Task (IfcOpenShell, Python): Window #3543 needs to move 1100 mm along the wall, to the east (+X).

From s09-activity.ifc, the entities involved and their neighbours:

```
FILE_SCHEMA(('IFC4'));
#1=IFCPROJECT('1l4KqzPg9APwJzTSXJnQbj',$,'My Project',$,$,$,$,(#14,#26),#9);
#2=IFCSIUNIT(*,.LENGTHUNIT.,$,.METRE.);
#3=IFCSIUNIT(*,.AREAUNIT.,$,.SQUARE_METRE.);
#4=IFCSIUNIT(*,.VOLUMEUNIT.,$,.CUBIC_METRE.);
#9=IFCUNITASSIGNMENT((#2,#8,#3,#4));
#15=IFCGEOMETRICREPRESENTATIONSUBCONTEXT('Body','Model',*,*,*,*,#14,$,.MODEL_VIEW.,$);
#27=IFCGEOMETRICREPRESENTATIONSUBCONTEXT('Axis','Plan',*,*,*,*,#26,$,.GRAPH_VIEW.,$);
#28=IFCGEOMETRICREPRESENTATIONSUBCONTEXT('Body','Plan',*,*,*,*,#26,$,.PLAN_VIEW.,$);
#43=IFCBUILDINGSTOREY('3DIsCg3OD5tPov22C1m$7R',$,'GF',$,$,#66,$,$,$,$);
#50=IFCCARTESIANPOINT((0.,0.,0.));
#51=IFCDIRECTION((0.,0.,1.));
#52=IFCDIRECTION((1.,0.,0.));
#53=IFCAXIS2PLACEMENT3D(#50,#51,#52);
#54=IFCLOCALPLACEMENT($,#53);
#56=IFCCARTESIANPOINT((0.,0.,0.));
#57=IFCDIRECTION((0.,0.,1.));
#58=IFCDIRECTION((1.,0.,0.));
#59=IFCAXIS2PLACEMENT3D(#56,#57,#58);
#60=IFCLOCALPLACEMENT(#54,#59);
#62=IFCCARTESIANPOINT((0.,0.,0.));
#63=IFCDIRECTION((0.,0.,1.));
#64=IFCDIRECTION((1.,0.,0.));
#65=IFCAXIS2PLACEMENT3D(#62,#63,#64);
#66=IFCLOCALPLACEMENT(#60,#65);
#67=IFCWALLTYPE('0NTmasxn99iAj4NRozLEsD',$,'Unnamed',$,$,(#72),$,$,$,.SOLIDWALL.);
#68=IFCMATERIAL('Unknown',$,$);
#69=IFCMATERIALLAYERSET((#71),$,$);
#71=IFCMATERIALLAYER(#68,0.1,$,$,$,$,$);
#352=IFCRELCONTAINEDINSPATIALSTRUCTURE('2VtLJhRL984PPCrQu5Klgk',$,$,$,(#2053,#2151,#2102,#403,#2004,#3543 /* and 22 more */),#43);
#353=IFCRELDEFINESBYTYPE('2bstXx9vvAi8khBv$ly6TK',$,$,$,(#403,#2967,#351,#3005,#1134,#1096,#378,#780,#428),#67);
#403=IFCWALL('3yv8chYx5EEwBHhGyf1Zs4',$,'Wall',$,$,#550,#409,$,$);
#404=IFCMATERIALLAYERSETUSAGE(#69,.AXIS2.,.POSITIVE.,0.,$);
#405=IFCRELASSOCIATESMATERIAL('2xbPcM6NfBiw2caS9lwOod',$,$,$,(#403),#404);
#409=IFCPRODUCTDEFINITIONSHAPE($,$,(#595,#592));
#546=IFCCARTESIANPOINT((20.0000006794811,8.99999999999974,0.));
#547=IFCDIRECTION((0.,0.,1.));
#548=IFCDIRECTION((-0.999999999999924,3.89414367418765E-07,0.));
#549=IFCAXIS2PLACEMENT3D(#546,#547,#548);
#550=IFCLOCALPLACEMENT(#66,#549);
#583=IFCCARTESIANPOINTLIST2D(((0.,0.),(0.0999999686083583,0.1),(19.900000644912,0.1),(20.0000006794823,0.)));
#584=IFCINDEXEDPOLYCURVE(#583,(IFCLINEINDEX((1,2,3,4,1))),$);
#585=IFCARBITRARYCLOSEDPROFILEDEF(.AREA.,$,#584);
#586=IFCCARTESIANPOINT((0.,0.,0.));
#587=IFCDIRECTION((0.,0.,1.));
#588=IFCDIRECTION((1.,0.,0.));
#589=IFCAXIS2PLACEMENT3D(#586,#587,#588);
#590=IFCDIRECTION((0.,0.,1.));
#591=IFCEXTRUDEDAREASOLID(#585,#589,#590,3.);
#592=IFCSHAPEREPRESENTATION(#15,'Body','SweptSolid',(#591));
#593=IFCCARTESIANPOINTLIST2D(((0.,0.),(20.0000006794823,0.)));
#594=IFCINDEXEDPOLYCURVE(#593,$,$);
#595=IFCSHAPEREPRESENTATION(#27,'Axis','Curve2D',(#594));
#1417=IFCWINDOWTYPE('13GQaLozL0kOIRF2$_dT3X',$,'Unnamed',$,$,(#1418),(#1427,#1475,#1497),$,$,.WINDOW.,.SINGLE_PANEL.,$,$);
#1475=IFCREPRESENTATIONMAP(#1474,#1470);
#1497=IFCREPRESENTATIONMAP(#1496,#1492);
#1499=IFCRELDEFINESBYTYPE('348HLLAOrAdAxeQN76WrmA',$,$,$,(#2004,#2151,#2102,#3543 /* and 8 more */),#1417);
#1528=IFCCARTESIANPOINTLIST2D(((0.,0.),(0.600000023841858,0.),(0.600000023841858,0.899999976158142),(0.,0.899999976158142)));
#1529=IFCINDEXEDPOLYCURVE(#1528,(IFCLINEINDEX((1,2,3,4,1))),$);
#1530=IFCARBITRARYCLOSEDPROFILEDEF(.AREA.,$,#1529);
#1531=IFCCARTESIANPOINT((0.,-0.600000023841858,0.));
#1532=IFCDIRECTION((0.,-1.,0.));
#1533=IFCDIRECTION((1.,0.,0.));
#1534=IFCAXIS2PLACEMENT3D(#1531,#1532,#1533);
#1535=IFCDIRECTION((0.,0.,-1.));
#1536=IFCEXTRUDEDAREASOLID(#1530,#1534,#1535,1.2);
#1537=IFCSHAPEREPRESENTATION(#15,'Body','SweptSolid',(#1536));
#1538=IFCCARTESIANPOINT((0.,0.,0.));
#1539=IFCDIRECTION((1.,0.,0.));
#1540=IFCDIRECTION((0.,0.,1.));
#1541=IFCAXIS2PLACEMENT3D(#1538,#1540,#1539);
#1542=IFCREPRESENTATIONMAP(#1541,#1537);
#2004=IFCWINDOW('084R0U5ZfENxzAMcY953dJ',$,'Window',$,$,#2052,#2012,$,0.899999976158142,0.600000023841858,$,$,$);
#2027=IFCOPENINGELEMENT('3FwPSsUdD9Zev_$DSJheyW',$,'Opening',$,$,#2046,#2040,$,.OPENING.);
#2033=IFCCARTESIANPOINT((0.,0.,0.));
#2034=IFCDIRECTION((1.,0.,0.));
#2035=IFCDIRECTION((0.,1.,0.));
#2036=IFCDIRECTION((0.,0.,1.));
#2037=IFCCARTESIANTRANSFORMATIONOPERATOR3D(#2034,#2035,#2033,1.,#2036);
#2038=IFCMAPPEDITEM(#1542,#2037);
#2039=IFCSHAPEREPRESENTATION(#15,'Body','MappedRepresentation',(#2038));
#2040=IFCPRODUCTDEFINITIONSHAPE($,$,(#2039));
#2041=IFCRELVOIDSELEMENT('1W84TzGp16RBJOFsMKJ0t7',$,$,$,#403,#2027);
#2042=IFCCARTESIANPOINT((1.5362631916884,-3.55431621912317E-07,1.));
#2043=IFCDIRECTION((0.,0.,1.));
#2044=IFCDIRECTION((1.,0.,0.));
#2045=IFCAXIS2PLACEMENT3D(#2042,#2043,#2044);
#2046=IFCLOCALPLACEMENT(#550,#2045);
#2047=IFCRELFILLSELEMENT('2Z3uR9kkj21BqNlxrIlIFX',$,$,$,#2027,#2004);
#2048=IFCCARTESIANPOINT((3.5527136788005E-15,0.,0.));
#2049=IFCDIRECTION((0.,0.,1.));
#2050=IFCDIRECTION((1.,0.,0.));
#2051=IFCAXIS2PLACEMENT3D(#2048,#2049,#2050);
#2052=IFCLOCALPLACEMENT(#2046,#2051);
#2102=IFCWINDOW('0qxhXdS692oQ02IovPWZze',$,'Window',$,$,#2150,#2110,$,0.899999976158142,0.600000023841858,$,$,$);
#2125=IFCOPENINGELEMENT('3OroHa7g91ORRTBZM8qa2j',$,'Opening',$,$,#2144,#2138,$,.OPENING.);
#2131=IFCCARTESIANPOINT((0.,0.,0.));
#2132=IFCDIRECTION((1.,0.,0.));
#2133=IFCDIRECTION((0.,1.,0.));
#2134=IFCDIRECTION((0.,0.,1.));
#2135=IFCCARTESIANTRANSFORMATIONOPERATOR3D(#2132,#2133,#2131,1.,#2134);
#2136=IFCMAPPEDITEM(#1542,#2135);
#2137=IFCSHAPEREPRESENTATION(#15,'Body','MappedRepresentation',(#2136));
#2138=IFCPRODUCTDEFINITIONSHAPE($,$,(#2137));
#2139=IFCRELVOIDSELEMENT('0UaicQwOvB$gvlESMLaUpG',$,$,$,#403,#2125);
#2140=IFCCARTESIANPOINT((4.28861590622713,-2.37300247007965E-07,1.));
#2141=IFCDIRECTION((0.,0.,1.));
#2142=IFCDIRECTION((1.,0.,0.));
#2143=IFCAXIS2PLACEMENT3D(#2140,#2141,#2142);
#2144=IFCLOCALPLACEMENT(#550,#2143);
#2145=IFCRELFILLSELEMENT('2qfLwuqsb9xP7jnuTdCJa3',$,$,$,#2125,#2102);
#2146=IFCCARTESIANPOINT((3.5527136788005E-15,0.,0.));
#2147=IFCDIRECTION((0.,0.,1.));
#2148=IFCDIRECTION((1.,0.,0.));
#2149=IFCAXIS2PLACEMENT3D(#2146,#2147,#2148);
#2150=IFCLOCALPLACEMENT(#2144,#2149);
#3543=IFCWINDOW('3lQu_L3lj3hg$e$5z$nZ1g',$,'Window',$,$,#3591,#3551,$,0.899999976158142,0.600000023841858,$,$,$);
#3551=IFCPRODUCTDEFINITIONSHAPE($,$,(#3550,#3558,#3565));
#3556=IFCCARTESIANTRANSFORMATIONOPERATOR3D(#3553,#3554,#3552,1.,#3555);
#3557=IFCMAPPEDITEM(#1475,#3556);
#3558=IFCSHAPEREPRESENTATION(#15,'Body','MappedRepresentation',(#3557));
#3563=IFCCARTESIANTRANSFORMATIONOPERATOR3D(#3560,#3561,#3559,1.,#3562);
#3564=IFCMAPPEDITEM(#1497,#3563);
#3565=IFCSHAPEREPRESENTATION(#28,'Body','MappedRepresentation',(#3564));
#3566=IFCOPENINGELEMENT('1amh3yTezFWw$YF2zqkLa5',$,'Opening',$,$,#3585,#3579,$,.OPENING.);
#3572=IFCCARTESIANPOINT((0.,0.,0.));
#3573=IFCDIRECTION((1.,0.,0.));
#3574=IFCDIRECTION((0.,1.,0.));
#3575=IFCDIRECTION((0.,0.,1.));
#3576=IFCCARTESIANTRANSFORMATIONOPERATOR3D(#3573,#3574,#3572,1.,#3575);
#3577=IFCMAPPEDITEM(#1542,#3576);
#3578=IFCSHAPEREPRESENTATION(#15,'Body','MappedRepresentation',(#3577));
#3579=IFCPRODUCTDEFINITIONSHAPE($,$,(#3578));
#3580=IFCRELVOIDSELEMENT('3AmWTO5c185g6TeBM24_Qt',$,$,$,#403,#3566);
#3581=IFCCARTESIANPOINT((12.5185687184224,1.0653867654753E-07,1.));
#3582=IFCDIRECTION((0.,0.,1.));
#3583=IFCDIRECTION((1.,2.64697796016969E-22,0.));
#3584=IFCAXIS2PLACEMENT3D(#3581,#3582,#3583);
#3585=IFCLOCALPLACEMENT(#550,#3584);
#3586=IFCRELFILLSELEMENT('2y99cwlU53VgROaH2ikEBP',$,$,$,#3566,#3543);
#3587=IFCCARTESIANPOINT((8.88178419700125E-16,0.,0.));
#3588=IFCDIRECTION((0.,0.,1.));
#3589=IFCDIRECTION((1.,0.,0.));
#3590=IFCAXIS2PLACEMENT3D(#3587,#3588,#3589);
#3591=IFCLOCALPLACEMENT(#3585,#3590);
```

```python
import ifcopenshell
import ifcopenshell.api.geometry
import ifcopenshell.util.placement
import ifcopenshell.util.unit

model = ifcopenshell.open("s09-activity.ifc")
unit_scale = ifcopenshell.util.unit.calculate_unit_scale(model)

window = model.by_guid("3lQu_L3lj3hg$e$5z$nZ1g")
opening = window.FillsVoids[0].RelatingOpeningElement
wall = opening.VoidsElements[0].RelatingBuildingElement

wall_matrix = ifcopenshell.util.placement.get_local_placement(wall.ObjectPlacement)
shift = wall_matrix[:3, 0] * -1.1 / unit_scale
before = ifcopenshell.util.placement.get_local_placement(window.ObjectPlacement)[:3, 3].copy()

# The window is placed relative to its opening, so it follows when the opening moves.
matrix = ifcopenshell.util.placement.get_local_placement(opening.ObjectPlacement)
matrix[:3, 3] += shift
ifcopenshell.api.geometry.edit_object_placement(
    model, product=opening, matrix=matrix, is_si=False, should_transform_children=True
)

after = ifcopenshell.util.placement.get_local_placement(window.ObjectPlacement)[:3, 3]
print("window moved by", (after - before).round(3) + 0.0)

model.write("s09-activity_updated.ifc")
```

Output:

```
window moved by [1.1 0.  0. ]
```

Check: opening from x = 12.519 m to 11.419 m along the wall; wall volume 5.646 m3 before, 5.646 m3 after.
